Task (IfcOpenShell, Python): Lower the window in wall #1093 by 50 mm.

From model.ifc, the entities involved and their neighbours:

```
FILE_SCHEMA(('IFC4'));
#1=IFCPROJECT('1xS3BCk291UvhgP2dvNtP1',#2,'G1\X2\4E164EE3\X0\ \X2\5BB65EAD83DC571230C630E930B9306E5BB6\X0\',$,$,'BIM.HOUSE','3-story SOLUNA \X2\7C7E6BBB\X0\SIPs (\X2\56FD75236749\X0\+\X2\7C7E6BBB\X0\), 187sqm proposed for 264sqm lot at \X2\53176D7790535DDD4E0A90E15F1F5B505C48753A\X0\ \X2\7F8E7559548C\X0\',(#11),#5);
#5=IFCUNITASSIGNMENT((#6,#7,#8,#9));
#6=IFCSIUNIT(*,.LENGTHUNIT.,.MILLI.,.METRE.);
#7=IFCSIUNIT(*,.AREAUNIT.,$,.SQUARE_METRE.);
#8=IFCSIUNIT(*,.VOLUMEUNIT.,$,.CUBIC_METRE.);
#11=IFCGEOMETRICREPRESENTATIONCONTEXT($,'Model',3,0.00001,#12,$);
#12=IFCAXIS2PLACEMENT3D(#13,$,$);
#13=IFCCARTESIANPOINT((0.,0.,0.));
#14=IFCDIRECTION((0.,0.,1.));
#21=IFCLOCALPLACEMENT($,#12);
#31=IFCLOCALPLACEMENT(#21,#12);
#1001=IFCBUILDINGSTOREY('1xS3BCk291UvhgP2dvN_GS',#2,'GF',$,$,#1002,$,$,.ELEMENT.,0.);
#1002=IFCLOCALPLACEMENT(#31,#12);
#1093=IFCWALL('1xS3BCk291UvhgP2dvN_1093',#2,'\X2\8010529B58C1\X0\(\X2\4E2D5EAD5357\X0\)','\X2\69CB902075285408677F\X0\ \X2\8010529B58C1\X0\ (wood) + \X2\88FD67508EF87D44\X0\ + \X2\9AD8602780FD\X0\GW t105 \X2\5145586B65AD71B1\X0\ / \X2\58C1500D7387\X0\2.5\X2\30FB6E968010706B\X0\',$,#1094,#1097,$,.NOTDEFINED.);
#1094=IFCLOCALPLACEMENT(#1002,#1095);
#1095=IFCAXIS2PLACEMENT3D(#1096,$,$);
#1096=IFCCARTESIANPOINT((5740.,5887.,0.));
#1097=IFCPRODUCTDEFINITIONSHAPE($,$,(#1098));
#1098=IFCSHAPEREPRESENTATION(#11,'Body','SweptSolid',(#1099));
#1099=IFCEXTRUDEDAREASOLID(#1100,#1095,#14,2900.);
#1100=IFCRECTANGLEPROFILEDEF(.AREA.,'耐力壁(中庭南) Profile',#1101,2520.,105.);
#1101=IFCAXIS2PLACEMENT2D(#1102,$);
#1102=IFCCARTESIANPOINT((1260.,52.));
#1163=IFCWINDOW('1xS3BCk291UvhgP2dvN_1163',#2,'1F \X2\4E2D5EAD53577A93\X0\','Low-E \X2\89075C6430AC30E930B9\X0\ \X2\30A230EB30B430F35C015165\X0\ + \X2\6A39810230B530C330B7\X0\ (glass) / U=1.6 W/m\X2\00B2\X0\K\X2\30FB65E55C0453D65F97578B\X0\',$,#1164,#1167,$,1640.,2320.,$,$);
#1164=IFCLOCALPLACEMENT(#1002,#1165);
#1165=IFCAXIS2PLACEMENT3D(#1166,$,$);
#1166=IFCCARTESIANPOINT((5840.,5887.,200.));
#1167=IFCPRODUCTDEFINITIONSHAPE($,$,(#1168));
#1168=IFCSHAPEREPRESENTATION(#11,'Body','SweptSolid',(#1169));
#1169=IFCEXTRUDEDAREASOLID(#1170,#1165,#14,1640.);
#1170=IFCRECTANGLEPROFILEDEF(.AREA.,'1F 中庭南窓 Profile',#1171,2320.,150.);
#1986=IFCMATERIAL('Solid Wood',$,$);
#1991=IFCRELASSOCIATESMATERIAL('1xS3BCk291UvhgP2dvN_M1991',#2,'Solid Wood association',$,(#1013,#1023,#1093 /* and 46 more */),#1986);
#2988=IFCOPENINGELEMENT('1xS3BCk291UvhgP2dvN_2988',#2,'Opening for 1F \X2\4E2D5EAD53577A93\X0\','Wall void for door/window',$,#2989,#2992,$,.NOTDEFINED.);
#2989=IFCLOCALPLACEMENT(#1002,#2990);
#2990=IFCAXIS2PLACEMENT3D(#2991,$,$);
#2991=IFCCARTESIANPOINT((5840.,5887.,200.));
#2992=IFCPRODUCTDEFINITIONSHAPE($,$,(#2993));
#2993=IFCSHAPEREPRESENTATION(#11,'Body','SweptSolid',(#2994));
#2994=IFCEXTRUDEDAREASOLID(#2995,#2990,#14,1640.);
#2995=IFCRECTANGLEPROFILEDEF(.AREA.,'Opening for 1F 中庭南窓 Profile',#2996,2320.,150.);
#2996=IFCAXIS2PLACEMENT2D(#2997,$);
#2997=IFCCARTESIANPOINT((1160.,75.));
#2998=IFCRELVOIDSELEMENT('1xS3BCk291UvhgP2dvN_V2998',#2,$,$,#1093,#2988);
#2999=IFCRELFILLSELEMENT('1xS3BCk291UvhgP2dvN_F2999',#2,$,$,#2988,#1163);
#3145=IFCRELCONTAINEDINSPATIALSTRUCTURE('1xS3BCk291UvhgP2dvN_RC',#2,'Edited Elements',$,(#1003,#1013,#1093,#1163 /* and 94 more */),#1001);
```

```python
import numpy as np
import ifcopenshell
import ifcopenshell.api.geometry
import ifcopenshell.util.placement
import ifcopenshell.util.unit

model = ifcopenshell.open("model.ifc")
unit_scale = ifcopenshell.util.unit.calculate_unit_scale(model)

window = model.by_guid("1xS3BCk291UvhgP2dvN_1163")
opening = window.FillsVoids[0].RelatingOpeningElement
dz = -0.05 / unit_scale

shift = np.array([0.0, 0.0, dz])
# The window is not placed relative to its opening, so move both.
for product in (opening, window):
    matrix = ifcopenshell.util.placement.get_local_placement(product.ObjectPlacement)
    matrix[:3, 3] += shift
    ifcopenshell.api.geometry.edit_object_placement(model, product=product, matrix=matrix, is_si=False)

print(f"moved by {dz * unit_scale:+.3f} m")

model.write("model_rev.ifc")
```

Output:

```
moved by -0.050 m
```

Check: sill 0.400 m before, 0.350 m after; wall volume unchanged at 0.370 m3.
